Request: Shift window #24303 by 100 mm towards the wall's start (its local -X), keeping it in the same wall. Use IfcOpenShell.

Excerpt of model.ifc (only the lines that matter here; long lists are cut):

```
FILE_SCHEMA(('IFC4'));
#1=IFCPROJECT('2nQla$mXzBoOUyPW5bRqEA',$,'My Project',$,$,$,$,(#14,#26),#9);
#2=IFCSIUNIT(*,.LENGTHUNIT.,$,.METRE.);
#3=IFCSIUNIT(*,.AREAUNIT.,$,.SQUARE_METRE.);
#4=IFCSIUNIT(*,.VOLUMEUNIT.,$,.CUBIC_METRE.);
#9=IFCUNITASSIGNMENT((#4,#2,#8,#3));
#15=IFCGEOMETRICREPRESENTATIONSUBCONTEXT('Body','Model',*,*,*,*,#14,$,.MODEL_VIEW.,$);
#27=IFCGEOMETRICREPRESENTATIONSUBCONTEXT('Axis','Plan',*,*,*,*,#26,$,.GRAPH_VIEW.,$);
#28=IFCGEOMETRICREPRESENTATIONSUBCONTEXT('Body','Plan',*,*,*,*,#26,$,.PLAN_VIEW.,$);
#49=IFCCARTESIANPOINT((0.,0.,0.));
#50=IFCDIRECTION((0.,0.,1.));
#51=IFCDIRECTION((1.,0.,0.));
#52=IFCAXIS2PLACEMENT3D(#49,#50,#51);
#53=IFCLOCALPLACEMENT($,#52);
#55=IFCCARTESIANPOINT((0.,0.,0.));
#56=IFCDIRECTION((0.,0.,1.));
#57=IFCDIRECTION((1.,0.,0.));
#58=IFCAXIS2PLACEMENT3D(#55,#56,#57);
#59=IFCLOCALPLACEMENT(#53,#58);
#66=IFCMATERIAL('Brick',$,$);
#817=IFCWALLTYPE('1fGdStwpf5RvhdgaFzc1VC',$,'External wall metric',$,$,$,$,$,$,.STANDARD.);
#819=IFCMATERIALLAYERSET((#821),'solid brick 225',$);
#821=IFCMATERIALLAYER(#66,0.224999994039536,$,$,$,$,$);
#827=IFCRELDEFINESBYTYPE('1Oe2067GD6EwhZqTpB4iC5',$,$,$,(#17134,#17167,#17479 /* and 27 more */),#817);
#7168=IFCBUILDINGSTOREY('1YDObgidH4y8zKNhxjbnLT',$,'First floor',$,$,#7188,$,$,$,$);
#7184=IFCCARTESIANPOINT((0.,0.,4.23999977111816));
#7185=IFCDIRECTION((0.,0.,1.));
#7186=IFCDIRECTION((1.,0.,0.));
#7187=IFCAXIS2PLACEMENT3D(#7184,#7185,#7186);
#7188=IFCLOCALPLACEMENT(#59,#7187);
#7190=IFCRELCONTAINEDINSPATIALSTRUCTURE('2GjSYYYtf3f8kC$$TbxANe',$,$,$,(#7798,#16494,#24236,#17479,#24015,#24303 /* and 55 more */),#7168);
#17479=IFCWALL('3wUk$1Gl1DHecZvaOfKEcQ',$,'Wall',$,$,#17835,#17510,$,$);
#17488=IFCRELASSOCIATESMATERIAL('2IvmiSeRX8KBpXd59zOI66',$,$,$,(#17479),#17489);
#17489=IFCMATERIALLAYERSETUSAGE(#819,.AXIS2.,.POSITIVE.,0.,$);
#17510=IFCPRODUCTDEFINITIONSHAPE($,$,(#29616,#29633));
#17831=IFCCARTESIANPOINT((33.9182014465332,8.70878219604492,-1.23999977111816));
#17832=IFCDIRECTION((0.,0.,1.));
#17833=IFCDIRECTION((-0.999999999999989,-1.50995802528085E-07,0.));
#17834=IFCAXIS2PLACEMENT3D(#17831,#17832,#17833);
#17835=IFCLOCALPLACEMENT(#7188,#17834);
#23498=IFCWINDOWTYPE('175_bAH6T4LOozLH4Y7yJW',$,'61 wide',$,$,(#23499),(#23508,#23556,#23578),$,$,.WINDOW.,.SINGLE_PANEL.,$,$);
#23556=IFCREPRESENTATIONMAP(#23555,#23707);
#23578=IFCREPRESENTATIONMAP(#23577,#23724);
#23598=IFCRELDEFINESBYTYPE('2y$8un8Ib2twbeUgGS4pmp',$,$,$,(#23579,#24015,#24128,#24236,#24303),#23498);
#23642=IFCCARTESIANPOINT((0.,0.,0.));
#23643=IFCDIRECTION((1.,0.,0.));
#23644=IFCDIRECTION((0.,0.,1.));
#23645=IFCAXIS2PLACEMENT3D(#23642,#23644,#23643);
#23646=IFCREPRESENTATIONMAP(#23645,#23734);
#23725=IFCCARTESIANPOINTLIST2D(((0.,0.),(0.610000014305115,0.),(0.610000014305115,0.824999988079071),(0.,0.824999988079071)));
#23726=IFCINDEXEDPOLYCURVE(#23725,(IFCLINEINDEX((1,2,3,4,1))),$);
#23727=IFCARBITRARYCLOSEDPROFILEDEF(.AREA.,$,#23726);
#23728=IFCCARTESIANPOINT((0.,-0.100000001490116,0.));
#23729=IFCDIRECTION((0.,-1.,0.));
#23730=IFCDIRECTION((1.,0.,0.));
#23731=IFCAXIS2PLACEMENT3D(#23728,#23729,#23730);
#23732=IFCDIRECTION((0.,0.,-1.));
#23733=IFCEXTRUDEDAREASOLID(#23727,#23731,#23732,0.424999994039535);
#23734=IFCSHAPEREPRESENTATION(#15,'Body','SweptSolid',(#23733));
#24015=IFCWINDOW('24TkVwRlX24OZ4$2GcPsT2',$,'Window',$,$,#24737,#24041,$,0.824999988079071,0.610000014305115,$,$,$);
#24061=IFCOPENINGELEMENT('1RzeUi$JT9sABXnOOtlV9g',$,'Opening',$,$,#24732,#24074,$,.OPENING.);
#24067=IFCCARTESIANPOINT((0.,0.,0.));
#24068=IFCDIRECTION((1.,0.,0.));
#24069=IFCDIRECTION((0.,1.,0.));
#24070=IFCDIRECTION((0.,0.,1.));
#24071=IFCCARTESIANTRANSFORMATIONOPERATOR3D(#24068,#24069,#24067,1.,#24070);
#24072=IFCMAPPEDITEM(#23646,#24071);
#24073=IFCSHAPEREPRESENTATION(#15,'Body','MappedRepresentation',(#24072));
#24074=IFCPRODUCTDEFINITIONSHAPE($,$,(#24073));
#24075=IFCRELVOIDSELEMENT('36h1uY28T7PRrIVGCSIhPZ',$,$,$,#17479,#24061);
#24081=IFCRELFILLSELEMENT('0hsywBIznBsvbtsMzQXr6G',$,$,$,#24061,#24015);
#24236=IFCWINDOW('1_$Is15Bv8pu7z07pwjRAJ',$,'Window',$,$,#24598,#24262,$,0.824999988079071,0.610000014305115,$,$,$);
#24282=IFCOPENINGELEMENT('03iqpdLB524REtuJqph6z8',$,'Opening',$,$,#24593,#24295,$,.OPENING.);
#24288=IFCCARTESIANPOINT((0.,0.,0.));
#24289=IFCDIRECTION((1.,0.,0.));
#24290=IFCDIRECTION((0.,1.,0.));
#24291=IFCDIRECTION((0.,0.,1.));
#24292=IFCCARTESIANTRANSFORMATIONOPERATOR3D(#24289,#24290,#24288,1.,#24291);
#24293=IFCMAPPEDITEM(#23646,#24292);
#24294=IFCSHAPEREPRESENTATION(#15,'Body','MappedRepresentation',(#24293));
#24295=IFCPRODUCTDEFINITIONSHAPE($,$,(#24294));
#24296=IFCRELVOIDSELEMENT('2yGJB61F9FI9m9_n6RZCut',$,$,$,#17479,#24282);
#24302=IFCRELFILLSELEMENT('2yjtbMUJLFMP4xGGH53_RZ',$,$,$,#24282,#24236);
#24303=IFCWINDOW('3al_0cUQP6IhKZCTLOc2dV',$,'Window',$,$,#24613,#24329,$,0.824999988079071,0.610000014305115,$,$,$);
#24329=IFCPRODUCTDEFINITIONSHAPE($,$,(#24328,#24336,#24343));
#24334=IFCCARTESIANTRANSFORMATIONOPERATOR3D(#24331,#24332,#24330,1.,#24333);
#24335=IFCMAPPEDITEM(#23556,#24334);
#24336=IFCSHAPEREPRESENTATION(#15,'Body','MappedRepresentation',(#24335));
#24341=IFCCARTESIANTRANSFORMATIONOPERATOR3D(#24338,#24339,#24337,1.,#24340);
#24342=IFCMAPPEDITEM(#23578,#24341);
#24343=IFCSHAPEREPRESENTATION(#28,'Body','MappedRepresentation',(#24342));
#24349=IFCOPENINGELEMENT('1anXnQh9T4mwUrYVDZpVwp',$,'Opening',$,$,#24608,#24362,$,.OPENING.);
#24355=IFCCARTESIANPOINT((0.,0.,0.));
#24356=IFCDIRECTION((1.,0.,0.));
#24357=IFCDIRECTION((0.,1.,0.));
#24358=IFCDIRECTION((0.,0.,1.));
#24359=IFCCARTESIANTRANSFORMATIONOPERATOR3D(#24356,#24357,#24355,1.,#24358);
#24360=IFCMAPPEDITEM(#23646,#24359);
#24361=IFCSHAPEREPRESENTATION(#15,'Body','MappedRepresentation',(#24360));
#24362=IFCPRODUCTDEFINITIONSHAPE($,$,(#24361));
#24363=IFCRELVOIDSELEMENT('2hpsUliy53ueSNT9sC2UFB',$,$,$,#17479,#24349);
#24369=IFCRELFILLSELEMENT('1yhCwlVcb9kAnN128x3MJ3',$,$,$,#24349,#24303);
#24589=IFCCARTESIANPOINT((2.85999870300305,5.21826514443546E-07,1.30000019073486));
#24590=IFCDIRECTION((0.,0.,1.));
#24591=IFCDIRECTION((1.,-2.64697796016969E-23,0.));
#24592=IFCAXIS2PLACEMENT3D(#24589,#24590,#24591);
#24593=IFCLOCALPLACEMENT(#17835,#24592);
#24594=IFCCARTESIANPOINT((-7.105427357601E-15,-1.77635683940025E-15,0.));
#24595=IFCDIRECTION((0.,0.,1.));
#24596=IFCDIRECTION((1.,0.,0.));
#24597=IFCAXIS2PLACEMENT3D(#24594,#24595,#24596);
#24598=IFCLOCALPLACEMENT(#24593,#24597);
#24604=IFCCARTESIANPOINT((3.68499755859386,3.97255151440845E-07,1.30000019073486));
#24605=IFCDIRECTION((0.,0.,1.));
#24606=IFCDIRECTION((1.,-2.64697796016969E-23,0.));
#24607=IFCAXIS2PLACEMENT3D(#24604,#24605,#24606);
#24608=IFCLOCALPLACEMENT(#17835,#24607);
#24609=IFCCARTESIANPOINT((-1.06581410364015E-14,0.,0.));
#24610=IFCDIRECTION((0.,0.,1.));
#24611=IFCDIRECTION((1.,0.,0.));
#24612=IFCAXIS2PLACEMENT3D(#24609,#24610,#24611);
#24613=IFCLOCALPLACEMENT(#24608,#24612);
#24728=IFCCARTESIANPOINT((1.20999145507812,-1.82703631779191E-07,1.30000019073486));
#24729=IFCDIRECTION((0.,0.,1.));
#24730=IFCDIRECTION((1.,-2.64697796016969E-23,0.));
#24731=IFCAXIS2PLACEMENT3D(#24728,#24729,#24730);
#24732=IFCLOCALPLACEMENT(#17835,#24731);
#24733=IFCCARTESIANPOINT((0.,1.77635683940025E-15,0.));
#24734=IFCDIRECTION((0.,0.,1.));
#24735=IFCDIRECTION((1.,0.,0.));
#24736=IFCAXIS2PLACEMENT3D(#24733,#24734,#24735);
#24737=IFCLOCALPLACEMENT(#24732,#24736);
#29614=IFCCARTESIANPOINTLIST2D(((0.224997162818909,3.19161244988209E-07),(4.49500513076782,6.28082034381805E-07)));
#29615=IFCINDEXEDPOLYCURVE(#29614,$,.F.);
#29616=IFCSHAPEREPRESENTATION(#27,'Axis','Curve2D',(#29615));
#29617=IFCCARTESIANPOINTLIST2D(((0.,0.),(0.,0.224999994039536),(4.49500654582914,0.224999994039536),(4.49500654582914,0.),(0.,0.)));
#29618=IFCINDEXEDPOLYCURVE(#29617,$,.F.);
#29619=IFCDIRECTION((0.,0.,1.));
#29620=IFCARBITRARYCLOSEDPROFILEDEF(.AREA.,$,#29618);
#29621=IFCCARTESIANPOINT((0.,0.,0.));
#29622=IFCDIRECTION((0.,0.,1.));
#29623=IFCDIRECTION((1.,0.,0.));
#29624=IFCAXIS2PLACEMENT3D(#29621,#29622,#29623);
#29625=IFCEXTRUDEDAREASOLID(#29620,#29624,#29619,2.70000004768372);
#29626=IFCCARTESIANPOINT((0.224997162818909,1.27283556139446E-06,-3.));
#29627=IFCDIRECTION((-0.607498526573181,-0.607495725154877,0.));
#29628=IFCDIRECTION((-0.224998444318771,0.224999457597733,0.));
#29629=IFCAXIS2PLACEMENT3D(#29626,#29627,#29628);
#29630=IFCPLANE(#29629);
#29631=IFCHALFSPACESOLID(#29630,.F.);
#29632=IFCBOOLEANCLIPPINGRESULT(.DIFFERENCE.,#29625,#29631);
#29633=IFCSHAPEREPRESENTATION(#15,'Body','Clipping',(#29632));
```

```python
import ifcopenshell
import ifcopenshell.api.geometry
import ifcopenshell.util.placement

model = ifcopenshell.open("model.ifc")

window = model.by_guid("3al_0cUQP6IhKZCTLOc2dV")
opening = window.FillsVoids[0].RelatingOpeningElement
wall = opening.VoidsElements[0].RelatingBuildingElement

wall_matrix = ifcopenshell.util.placement.get_local_placement(wall.ObjectPlacement)
shift = wall_matrix[:3, 0] * -0.1
before = ifcopenshell.util.placement.get_local_placement(window.ObjectPlacement)[:3, 3].copy()

# The window is placed relative to its opening, so it follows when the opening moves.
matrix = ifcopenshell.util.placement.get_local_placement(opening.ObjectPlacement)
matrix[:3, 3] += shift
ifcopenshell.api.geometry.edit_object_placement(
    model, product=opening, matrix=matrix, is_si=False, should_transform_children=True
)

after = ifcopenshell.util.placement.get_local_placement(window.ObjectPlacement)[:3, 3]
print("window moved by", (after - before).round(3) + 0.0)

model.write("model_rev.ifc")
```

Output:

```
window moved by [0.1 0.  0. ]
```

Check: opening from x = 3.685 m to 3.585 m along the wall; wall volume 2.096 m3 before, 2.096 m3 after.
